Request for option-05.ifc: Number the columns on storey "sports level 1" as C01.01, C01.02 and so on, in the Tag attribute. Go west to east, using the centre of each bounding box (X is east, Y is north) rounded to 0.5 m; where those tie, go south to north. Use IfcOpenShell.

First a look at what the model holds.

```python
import ifcopenshell
import ifcopenshell.util.element
import ifcopenshell.util.placement

model = ifcopenshell.open("option-05.ifc")
print(model.schema)
storey = next(s for s in model.by_type("IfcBuildingStorey") if s.Name == "sports level 1")
columns = [e for e in ifcopenshell.util.element.get_decomposition(storey) if e.is_a("IfcColumn")]
for e in sorted(columns, key=lambda e: e.id()):
    origin = ifcopenshell.util.placement.get_local_placement(e.ObjectPlacement)[:3, 3]
    print(e.id(), e.Tag, e.Name, origin.round(2) + 0.0, sep=" | ")
```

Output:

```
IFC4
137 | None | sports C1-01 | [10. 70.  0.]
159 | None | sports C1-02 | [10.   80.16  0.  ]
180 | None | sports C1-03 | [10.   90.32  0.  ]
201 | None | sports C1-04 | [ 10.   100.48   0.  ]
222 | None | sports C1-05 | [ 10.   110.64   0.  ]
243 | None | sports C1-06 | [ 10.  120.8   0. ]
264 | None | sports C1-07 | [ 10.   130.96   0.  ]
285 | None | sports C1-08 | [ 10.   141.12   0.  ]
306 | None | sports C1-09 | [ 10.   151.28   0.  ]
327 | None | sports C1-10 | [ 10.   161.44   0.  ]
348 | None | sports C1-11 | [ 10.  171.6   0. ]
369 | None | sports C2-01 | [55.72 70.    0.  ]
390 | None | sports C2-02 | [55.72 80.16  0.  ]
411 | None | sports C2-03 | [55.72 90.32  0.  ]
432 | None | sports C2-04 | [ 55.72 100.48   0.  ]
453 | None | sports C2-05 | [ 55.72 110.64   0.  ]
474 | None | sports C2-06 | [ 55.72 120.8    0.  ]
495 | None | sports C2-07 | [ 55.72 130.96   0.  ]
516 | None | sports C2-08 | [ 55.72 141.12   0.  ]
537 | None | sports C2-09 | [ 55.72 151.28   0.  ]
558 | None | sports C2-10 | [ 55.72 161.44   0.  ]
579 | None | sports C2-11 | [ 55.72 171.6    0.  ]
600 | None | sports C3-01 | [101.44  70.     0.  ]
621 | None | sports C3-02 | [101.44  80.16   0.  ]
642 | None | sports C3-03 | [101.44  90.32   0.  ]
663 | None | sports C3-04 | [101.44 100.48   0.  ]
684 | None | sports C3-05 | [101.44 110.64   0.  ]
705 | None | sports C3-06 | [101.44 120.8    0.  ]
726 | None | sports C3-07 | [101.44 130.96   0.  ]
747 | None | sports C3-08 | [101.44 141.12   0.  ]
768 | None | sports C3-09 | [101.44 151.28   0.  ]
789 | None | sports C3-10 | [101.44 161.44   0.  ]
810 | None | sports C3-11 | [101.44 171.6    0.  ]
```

```python
import ifcopenshell
import ifcopenshell.geom
import ifcopenshell.util.element
import ifcopenshell.util.shape

model = ifcopenshell.open("option-05.ifc")
settings = ifcopenshell.geom.settings()
settings.set("use-world-coords", True)


def centre(element):
    shape = ifcopenshell.geom.create_shape(settings, element)
    return ifcopenshell.util.shape.get_bbox_centroid(shape.geometry)


storey = next(s for s in model.by_type("IfcBuildingStorey") if s.Name == "sports level 1")
columns = [e for e in ifcopenshell.util.element.get_decomposition(storey) if e.is_a("IfcColumn")]

# Insertion points can sit at a corner or the storey origin, so sort by the geometry (in metres).
centres = {e: centre(e) for e in columns}
columns.sort(key=lambda e: (round(centres[e][0] / 0.5), centres[e][1]))

for i, e in enumerate(columns, start=1):
    number = f"C01.{i:02d}"
    e.Tag = number
    print(e.id(), number)

model.write("option-05-out.ifc")
```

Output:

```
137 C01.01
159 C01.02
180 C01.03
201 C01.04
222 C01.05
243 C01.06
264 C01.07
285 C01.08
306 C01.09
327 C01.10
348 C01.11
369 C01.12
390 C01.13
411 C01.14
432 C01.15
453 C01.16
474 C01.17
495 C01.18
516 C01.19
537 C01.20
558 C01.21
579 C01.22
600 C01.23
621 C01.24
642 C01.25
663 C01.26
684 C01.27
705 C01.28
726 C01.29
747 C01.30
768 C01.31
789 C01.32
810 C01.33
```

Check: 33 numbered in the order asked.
